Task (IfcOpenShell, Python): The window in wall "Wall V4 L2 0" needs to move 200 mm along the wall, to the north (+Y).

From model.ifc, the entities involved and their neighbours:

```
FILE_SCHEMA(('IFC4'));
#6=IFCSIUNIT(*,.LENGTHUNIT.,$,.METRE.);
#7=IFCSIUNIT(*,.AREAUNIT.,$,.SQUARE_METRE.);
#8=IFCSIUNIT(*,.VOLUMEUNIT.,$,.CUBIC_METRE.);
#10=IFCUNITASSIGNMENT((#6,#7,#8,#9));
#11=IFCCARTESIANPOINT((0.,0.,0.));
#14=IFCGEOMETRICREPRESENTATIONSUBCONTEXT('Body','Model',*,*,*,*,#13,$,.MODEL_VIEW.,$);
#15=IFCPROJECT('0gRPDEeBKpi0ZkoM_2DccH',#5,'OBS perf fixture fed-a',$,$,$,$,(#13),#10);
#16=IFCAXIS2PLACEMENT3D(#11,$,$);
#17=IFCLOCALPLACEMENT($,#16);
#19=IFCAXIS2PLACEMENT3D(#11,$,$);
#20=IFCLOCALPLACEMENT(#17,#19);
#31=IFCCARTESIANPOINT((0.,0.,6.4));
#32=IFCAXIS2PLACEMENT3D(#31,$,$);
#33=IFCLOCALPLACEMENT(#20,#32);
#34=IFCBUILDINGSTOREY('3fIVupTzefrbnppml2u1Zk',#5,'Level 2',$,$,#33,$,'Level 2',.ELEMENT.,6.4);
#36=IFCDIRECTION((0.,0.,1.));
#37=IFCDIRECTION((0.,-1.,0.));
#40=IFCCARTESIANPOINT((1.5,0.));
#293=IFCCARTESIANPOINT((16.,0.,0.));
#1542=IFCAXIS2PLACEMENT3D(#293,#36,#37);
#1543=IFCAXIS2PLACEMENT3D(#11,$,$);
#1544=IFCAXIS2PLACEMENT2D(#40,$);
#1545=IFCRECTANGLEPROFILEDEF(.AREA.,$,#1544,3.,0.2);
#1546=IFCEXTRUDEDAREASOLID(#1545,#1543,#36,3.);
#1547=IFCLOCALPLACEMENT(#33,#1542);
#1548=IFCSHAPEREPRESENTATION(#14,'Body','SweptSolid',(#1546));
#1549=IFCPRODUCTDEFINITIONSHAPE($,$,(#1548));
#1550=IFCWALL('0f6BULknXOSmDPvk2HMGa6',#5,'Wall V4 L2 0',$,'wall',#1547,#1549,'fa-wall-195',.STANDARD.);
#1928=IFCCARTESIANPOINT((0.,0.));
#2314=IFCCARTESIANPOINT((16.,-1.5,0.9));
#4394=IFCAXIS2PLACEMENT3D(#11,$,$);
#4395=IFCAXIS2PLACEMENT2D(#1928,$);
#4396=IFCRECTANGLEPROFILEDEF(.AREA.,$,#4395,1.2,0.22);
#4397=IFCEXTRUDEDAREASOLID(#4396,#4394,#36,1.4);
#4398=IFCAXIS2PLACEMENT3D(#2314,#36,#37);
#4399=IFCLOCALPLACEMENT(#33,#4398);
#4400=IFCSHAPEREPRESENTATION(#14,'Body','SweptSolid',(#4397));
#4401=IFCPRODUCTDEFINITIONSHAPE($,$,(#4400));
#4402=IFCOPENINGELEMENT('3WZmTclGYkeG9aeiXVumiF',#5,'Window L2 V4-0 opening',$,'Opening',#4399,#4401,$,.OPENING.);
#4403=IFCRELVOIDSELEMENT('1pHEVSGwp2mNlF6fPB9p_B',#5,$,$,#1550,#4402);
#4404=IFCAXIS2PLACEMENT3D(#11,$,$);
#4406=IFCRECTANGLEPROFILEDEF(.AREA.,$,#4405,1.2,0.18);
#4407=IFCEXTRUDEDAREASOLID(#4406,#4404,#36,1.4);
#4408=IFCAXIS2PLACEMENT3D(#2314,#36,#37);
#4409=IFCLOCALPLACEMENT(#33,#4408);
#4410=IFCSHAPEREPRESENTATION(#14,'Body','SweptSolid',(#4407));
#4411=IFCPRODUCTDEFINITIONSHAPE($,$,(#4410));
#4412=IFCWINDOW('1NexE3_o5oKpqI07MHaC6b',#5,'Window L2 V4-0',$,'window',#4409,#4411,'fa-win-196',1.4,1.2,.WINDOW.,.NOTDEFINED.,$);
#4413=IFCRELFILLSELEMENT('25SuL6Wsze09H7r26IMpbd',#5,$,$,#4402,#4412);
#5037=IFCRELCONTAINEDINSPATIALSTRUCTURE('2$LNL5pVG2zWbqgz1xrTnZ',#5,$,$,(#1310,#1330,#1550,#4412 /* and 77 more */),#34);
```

```python
import ifcopenshell
import ifcopenshell.api.geometry
import ifcopenshell.util.placement
import ifcopenshell.util.unit

model = ifcopenshell.open("model.ifc")
unit_scale = ifcopenshell.util.unit.calculate_unit_scale(model)

window = model.by_guid("1NexE3_o5oKpqI07MHaC6b")
opening = window.FillsVoids[0].RelatingOpeningElement
wall = opening.VoidsElements[0].RelatingBuildingElement

wall_matrix = ifcopenshell.util.placement.get_local_placement(wall.ObjectPlacement)
shift = wall_matrix[:3, 0] * -0.2 / unit_scale
before = ifcopenshell.util.placement.get_local_placement(window.ObjectPlacement)[:3, 3].copy()

# The window is not placed relative to its opening, so move both.
for product in (opening, window):
    matrix = ifcopenshell.util.placement.get_local_placement(product.ObjectPlacement)
    matrix[:3, 3] += shift
    ifcopenshell.api.geometry.edit_object_placement(model, product=product, matrix=matrix, is_si=False)

after = ifcopenshell.util.placement.get_local_placement(window.ObjectPlacement)[:3, 3]
print("window moved by", (after - before).round(3) + 0.0)

model.write("model_v2.ifc")
```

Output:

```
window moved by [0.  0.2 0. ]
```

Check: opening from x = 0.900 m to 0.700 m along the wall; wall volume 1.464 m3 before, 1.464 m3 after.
